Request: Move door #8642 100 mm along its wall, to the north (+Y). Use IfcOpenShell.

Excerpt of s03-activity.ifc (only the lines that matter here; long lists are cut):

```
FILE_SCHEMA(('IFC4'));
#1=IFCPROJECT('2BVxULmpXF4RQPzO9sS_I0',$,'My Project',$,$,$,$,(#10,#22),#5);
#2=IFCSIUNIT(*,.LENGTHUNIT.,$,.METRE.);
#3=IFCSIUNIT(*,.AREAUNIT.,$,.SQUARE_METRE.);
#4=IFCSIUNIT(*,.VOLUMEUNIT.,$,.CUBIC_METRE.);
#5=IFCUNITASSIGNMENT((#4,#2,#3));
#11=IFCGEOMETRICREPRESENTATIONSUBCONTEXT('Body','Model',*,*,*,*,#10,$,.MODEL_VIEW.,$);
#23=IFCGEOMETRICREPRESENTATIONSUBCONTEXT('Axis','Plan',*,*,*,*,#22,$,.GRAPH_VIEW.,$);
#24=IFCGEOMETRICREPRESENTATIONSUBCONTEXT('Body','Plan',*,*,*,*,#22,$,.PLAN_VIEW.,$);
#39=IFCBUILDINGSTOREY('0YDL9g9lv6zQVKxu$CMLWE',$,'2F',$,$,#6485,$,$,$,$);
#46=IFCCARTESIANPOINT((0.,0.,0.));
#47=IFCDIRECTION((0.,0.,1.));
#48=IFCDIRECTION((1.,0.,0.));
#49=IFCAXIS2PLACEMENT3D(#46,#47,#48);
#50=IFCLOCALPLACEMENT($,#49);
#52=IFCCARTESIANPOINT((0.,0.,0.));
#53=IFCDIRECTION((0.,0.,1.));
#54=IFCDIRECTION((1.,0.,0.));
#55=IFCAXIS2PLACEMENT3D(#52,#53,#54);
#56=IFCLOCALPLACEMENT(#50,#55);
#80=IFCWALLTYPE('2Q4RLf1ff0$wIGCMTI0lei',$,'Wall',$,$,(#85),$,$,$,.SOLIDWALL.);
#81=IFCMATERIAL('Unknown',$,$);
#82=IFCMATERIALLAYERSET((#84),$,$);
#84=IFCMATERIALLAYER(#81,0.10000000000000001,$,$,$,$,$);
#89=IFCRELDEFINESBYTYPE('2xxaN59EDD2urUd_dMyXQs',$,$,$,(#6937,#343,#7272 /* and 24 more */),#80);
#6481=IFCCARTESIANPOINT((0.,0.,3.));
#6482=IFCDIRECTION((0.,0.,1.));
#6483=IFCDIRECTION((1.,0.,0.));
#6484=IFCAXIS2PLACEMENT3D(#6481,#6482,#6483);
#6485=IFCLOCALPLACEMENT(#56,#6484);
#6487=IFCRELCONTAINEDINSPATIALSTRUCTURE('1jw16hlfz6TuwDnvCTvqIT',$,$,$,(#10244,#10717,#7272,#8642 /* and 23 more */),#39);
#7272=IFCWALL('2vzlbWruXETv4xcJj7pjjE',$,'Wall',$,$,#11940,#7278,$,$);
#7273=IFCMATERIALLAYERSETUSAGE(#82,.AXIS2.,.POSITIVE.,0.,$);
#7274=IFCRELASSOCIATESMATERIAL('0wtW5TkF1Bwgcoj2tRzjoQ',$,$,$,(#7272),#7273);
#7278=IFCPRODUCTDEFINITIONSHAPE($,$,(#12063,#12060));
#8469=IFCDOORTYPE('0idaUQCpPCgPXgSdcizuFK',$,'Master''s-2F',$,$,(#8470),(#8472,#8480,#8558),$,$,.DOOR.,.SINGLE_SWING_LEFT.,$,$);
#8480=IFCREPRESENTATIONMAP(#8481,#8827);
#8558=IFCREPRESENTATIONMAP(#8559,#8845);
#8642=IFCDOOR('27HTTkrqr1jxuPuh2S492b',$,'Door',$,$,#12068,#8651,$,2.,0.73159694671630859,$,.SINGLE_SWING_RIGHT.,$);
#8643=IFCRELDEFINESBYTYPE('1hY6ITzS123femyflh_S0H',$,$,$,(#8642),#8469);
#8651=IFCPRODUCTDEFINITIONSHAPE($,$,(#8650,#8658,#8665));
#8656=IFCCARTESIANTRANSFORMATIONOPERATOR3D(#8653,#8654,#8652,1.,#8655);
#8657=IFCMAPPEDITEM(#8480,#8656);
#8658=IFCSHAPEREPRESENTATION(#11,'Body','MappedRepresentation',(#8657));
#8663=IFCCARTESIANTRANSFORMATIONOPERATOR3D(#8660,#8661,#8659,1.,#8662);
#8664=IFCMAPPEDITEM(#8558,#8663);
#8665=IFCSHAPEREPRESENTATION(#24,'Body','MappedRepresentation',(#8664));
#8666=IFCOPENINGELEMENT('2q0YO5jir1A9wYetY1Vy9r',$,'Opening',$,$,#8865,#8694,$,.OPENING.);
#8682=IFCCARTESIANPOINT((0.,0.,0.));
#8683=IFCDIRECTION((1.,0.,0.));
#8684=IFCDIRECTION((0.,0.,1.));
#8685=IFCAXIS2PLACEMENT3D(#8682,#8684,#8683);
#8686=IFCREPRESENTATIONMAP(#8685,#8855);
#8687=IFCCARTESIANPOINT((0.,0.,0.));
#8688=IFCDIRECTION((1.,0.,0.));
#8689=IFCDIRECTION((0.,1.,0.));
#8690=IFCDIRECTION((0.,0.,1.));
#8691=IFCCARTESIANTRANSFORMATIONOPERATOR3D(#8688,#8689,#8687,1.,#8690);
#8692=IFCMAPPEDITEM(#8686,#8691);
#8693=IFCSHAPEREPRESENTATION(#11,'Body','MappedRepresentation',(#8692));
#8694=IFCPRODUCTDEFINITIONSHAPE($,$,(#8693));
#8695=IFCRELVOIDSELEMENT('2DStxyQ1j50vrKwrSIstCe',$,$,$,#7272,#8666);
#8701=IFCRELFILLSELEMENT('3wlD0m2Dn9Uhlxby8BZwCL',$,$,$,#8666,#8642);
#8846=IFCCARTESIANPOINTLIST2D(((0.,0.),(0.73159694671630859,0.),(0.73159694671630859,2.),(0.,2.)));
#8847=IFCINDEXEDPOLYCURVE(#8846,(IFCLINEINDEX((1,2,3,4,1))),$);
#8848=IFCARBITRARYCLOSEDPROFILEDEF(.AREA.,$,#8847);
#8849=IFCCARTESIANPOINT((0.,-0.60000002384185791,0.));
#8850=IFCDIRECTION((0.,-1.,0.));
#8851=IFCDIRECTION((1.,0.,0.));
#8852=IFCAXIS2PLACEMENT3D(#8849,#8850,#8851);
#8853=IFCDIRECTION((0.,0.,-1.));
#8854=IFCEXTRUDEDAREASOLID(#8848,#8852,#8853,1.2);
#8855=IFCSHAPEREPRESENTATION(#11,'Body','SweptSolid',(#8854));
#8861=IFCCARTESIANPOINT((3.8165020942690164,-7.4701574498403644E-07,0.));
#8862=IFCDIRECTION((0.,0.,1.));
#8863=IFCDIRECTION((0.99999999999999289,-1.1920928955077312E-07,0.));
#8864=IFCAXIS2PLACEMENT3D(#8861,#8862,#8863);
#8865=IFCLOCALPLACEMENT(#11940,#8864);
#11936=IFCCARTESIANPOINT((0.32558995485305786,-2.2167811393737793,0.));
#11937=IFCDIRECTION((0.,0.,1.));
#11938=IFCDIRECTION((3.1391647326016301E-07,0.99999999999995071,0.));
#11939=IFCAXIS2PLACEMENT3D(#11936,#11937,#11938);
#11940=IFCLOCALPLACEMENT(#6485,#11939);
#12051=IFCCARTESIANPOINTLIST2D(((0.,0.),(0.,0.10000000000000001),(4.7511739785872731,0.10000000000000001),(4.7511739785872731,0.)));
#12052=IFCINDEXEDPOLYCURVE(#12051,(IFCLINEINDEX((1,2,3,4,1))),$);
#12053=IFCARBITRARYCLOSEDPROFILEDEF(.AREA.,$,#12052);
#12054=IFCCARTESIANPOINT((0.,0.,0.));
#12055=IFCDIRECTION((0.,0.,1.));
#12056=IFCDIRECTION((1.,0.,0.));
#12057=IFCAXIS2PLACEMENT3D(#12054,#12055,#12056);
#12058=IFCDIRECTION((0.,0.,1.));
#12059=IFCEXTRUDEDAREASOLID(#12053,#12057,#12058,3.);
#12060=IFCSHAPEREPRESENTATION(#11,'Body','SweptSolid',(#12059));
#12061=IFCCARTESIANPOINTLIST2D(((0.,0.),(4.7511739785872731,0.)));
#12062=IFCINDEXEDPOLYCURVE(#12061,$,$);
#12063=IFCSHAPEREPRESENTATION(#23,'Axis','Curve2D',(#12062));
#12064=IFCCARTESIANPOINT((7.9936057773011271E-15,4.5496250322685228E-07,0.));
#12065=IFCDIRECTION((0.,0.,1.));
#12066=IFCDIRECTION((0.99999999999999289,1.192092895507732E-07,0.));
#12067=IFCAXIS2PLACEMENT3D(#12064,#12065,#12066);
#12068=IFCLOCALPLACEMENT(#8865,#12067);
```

```python
import ifcopenshell
import ifcopenshell.api.geometry
import ifcopenshell.util.placement

model = ifcopenshell.open("s03-activity.ifc")

door = model.by_guid("27HTTkrqr1jxuPuh2S492b")
opening = door.FillsVoids[0].RelatingOpeningElement
wall = opening.VoidsElements[0].RelatingBuildingElement

wall_matrix = ifcopenshell.util.placement.get_local_placement(wall.ObjectPlacement)
shift = wall_matrix[:3, 0] * 0.1
before = ifcopenshell.util.placement.get_local_placement(door.ObjectPlacement)[:3, 3].copy()

# The door is placed relative to its opening, so it follows when the opening moves.
matrix = ifcopenshell.util.placement.get_local_placement(opening.ObjectPlacement)
matrix[:3, 3] += shift
ifcopenshell.api.geometry.edit_object_placement(
    model, product=opening, matrix=matrix, is_si=False, should_transform_children=True
)

after = ifcopenshell.util.placement.get_local_placement(door.ObjectPlacement)[:3, 3]
print("door moved by", (after - before).round(3) + 0.0)

model.write("s03-activity_updated.ifc")
```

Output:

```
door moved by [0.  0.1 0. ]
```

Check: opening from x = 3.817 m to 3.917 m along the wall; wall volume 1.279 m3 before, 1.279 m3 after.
